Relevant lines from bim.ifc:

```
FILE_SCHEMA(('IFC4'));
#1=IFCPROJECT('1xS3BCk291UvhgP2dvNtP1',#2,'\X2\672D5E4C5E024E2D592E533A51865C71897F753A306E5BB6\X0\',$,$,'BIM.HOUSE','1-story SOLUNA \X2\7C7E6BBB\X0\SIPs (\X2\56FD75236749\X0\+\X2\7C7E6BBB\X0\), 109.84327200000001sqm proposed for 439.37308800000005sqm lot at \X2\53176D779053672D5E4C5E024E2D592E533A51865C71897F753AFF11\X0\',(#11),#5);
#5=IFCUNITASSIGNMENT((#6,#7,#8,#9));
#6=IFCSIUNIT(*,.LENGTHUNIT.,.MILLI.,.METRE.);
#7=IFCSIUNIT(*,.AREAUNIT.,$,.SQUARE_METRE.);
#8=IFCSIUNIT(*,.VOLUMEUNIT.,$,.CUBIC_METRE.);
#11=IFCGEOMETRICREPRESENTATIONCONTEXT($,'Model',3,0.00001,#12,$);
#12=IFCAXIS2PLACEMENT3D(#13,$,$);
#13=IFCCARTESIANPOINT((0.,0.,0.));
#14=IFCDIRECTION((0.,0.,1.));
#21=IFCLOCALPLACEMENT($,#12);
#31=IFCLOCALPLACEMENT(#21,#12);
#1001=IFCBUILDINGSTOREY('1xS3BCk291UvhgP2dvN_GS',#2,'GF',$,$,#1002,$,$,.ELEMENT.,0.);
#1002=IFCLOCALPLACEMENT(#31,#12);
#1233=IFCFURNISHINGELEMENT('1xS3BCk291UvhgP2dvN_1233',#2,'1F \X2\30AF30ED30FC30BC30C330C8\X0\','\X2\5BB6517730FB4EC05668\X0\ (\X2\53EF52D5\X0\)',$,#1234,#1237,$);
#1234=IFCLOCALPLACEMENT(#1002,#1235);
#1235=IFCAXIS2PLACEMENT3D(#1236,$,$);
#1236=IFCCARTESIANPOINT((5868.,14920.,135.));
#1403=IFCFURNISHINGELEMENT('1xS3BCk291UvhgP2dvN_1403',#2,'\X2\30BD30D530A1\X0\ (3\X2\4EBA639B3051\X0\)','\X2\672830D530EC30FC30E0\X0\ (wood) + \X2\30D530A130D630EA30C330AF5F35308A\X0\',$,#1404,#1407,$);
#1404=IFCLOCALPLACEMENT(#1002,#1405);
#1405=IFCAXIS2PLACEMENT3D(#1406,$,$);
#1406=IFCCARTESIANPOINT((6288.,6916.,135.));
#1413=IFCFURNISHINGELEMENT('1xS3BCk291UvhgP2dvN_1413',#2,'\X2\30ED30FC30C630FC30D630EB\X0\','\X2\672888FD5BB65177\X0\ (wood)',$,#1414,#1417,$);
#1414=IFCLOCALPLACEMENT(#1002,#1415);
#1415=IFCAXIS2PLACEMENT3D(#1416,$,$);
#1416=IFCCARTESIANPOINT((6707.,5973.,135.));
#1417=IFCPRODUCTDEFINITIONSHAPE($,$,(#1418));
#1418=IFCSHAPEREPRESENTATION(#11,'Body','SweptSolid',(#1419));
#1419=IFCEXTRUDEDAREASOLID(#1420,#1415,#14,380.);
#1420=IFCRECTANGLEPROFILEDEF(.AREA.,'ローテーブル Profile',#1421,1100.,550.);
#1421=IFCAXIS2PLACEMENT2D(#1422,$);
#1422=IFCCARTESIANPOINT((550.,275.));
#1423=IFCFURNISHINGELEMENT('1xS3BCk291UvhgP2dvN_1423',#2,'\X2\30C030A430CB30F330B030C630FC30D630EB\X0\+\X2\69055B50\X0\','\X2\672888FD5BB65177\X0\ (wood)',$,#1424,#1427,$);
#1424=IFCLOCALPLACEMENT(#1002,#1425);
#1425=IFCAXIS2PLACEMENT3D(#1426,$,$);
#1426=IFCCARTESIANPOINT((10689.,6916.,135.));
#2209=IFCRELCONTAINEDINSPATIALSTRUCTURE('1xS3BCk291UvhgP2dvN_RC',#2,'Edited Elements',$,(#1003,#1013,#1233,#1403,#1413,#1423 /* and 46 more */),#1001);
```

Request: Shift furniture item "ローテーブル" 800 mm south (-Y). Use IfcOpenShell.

```python
import ifcopenshell
import ifcopenshell.api.geometry
import ifcopenshell.util.placement

model = ifcopenshell.open("bim.ifc")

item = model.by_guid("1xS3BCk291UvhgP2dvN_1413")
matrix = ifcopenshell.util.placement.get_local_placement(item.ObjectPlacement)
matrix[1, 3] -= 800.0
ifcopenshell.api.geometry.edit_object_placement(model, product=item, matrix=matrix, is_si=False)

print(ifcopenshell.util.placement.get_local_placement(item.ObjectPlacement).round(3) + 0.0)

model.write("bim-out.ifc")
```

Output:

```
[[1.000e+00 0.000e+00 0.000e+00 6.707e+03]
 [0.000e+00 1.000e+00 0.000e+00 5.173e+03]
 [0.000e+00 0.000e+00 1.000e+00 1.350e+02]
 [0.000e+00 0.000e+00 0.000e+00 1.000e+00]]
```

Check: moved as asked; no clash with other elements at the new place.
